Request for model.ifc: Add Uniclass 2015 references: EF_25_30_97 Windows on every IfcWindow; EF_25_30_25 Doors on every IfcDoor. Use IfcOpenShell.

First a look at what the model holds.

```python
import ifcopenshell

model = ifcopenshell.open("model.ifc")
print(model.schema)
print("classifications:", [c.Name for c in model.by_type("IfcClassification")])
for ifc_class in ("IfcDoor", "IfcRoof", "IfcStair", "IfcWall", "IfcWindow"):
    print(ifc_class, len(model.by_type(ifc_class)))
```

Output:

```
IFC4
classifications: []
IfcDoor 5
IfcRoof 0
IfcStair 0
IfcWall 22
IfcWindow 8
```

```python
import ifcopenshell
import ifcopenshell.api.classification

model = ifcopenshell.open("model.ifc")

system = ifcopenshell.api.classification.add_classification(model, classification="Uniclass 2015")

codes = {
    "IfcWindow": ("EF_25_30_97", "Windows"),
    "IfcDoor": ("EF_25_30_25", "Doors"),
}
for ifc_class, (code, name) in codes.items():
    products = model.by_type(ifc_class)
    ifcopenshell.api.classification.add_reference(
        model, products=products, classification=system, identification=code, name=name
    )
    print(code, len(products))

model.write("model_edited.ifc")
```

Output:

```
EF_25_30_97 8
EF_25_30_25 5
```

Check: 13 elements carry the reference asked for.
